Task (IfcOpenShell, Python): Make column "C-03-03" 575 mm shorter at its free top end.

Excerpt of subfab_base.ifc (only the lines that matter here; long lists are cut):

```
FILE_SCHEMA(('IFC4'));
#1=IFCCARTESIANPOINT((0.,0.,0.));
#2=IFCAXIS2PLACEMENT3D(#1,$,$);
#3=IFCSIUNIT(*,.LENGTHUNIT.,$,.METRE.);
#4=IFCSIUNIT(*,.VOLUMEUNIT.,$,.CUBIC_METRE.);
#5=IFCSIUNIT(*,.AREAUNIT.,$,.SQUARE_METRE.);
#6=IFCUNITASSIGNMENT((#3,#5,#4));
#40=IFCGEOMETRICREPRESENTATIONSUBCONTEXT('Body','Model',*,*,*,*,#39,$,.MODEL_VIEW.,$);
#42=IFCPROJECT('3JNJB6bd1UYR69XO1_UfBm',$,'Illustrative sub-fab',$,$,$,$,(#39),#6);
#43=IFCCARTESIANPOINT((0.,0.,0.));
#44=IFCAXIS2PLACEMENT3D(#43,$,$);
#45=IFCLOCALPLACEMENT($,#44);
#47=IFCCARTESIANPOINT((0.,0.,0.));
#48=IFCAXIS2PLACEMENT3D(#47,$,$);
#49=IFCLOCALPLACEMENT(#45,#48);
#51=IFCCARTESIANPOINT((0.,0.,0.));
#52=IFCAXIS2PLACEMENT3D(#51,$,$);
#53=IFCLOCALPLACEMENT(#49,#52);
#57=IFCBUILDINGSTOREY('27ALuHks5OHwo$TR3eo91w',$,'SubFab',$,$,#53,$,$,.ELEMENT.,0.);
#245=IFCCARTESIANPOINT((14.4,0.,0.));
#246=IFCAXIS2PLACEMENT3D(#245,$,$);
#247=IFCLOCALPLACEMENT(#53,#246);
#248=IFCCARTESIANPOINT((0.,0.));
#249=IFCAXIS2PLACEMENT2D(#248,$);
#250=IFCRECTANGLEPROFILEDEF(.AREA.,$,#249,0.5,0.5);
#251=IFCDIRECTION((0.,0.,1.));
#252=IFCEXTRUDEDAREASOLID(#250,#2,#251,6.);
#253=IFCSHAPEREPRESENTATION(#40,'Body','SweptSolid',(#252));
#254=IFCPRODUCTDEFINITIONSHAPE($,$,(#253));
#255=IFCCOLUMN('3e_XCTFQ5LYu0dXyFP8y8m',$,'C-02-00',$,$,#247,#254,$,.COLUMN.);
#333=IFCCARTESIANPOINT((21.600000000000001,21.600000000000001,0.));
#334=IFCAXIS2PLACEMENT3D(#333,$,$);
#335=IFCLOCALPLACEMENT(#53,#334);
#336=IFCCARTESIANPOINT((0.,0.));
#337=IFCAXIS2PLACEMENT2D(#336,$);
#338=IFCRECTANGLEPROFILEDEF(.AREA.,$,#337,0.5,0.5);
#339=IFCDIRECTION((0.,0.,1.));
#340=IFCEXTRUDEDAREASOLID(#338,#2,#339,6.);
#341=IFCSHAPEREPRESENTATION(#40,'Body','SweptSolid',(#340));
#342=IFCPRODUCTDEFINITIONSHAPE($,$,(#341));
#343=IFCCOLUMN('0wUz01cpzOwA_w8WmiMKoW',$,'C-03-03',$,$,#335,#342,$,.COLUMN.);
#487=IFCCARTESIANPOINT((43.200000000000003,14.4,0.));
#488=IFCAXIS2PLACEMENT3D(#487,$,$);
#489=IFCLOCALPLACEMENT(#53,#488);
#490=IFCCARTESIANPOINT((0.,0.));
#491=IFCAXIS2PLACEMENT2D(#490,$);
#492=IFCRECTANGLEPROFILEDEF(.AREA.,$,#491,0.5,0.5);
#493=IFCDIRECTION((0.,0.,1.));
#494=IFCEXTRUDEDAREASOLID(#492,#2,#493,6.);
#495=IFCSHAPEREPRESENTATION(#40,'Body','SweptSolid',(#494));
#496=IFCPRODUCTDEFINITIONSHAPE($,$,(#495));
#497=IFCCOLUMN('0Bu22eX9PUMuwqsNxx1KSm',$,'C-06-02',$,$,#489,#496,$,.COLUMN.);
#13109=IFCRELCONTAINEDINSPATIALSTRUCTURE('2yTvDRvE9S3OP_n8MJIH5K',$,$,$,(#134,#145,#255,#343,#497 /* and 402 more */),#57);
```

```python
import ifcopenshell
import ifcopenshell.util.representation

model = ifcopenshell.open("subfab_base.ifc")

member = model.by_guid("0wUz01cpzOwA_w8WmiMKoW")
change = -0.575

# The extrusion runs towards the end named, so only its depth changes.
body = ifcopenshell.util.representation.get_representation(member, "Model", "Body")
solid = body.Items[0]
old_length = solid.Depth
solid.Depth += change

print(f"length {old_length:g} -> {solid.Depth:g}")

model.write("subfab_base_edited.ifc")
```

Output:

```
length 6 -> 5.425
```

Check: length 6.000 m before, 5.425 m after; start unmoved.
